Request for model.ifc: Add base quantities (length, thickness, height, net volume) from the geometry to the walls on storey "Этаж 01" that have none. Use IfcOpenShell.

First a look at what the model holds.

```python
import ifcopenshell
import ifcopenshell.util.element
import ifcopenshell.util.unit

model = ifcopenshell.open("model.ifc")
print(model.schema)
for unit_type in ("LENGTHUNIT", "AREAUNIT", "VOLUMEUNIT"):
    print(unit_type, ifcopenshell.util.unit.calculate_unit_scale(model, unit_type))
storey = next(s for s in model.by_type("IfcBuildingStorey") if s.Name == "Этаж 01")
walls = [e for e in ifcopenshell.util.element.get_decomposition(storey) if e.is_a("IfcWall")]
for e in sorted(walls, key=lambda e: e.id()):
    print(e.id(), e.is_a(), e.Name, list(ifcopenshell.util.element.get_psets(e, qtos_only=True)), sep=" | ")
```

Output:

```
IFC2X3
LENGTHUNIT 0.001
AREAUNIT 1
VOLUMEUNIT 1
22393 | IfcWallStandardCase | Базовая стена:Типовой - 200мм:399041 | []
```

```python
import ifcopenshell
import ifcopenshell.api.pset
import ifcopenshell.geom
import ifcopenshell.util.element
import ifcopenshell.util.shape
import ifcopenshell.util.unit

model = ifcopenshell.open("model.ifc")
unit_scale = ifcopenshell.util.unit.calculate_unit_scale(model)
volume_scale = ifcopenshell.util.unit.calculate_unit_scale(model, "VOLUMEUNIT")
settings = ifcopenshell.geom.settings()

storey = next(s for s in model.by_type("IfcBuildingStorey") if s.Name == "Этаж 01")
walls = [e for e in ifcopenshell.util.element.get_decomposition(storey) if e.is_a("IfcWall")]

for e in sorted(walls, key=lambda e: e.id()):
    if ifcopenshell.util.element.get_psets(e, qtos_only=True, should_inherit=False):
        continue
    # Geometry comes back in metres, in the element's own axes.
    shape = ifcopenshell.geom.create_shape(settings, e)
    values = {
        "Length": ifcopenshell.util.shape.get_x(shape.geometry) / unit_scale,
        "Width": ifcopenshell.util.shape.get_y(shape.geometry) / unit_scale,
        "Height": ifcopenshell.util.shape.get_z(shape.geometry) / unit_scale,
        "NetVolume": ifcopenshell.util.shape.get_volume(shape.geometry) / volume_scale,
    }
    qto = ifcopenshell.api.pset.add_qto(model, product=e, name="BaseQuantities")
    ifcopenshell.api.pset.edit_qto(model, qto=qto, properties=values)
    print(e.id(), {k: round(v, 3) for k, v in values.items()})

model.write("model_updated.ifc")
```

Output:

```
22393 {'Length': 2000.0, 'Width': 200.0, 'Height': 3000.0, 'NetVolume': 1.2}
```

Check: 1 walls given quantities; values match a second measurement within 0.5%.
